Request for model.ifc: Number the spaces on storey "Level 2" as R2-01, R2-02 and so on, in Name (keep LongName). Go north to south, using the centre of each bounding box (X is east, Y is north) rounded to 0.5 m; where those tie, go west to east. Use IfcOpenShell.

First a look at what the model holds.

```python
import ifcopenshell
import ifcopenshell.util.element
import ifcopenshell.util.placement

model = ifcopenshell.open("model.ifc")
print(model.schema)
storey = next(s for s in model.by_type("IfcBuildingStorey") if s.Name == "Level 2")
spaces = [e for e in ifcopenshell.util.element.get_decomposition(storey) if e.is_a("IfcSpace")]
for e in sorted(spaces, key=lambda e: e.id()):
    origin = ifcopenshell.util.placement.get_local_placement(e.ObjectPlacement)[:3, 3]
    print(e.id(), e.Name, e.LongName, origin.round(2) + 0.0, sep=" | ")
```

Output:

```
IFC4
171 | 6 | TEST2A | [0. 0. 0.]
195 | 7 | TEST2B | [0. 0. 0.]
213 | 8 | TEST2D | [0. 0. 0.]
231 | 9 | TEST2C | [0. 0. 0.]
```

```python
import ifcopenshell
import ifcopenshell.geom
import ifcopenshell.util.element
import ifcopenshell.util.shape

model = ifcopenshell.open("model.ifc")
settings = ifcopenshell.geom.settings()
settings.set("use-world-coords", True)


def centre(element):
    shape = ifcopenshell.geom.create_shape(settings, element)
    return ifcopenshell.util.shape.get_bbox_centroid(shape.geometry)


storey = next(s for s in model.by_type("IfcBuildingStorey") if s.Name == "Level 2")
spaces = [e for e in ifcopenshell.util.element.get_decomposition(storey) if e.is_a("IfcSpace")]

# Insertion points can sit at a corner or the storey origin, so sort by the geometry (in metres).
centres = {e: centre(e) for e in spaces}
spaces.sort(key=lambda e: (-round(centres[e][1] / 0.5), centres[e][0]))

for i, e in enumerate(spaces, start=1):
    number = f"R2-{i:02d}"
    e.Name = number
    print(e.id(), number)

model.write("model_v2.ifc")
```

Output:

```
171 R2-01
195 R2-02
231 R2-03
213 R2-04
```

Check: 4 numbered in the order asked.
